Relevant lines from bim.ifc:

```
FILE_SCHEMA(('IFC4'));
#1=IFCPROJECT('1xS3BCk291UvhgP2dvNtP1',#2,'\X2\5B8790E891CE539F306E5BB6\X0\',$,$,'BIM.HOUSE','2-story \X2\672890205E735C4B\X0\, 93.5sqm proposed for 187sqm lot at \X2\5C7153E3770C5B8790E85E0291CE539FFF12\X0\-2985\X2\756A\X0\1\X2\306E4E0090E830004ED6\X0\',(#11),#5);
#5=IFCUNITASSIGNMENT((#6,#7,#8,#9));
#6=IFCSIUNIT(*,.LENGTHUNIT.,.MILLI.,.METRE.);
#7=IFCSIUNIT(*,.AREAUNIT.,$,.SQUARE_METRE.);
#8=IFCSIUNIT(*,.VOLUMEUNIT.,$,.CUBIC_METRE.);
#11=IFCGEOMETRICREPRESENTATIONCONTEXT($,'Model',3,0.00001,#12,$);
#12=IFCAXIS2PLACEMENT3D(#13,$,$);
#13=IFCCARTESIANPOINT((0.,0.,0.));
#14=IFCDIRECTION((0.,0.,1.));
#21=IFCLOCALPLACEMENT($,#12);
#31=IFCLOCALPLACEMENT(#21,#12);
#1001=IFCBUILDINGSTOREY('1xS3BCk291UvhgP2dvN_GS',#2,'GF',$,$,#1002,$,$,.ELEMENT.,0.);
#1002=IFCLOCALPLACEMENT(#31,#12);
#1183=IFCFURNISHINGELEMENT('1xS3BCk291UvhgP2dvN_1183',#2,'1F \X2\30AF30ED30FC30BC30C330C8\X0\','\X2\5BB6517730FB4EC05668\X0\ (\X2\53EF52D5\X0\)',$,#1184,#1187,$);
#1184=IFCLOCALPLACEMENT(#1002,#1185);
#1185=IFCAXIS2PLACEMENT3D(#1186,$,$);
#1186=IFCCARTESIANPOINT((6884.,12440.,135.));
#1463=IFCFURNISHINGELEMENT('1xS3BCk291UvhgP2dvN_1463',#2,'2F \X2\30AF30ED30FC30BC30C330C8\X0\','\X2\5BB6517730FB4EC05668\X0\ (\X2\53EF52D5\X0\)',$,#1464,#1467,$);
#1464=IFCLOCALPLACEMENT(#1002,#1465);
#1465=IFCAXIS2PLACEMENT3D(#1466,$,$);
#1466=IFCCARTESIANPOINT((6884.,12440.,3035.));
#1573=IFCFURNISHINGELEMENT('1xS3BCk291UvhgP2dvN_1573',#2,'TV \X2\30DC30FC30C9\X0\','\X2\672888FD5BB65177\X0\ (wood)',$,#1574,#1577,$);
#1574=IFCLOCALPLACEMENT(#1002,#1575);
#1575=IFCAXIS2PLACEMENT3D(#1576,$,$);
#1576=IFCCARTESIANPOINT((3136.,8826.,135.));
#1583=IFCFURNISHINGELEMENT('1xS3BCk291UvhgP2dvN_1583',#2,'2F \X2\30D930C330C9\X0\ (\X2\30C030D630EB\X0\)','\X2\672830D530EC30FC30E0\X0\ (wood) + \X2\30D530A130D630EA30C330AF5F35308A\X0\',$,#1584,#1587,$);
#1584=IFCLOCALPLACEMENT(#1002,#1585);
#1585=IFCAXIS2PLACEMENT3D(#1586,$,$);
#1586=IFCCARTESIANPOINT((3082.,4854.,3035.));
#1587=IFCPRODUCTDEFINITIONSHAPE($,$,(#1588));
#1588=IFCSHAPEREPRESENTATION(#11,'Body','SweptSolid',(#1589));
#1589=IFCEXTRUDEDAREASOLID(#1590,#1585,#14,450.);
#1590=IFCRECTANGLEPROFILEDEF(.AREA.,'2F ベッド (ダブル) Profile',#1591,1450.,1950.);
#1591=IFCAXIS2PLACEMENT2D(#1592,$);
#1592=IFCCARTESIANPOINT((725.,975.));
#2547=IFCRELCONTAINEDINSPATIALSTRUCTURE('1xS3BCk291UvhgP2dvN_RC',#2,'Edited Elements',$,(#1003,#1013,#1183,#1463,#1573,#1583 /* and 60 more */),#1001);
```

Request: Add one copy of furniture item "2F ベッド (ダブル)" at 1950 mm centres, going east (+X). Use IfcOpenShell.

```python
import numpy as np
import ifcopenshell
import ifcopenshell.api.geometry
import ifcopenshell.api.root
import ifcopenshell.util.element
import ifcopenshell.util.placement

model = ifcopenshell.open("bim.ifc")


def reuse_history(source, copy):
    """copy_class also copies each property set's owner history, people and application; keep the originals."""
    for rel in copy.IsDefinedBy:
        if rel.is_a("IfcRelDefinesByProperties") and (history := rel.RelatingPropertyDefinition.OwnerHistory):
            rel.RelatingPropertyDefinition.OwnerHistory = source.OwnerHistory
            ifcopenshell.util.element.remove_deep2(model, history)


source = model.by_guid("1xS3BCk291UvhgP2dvN_1583")
base = ifcopenshell.util.placement.get_local_placement(source.ObjectPlacement)
step = np.array([1.0, 0.0, 0.0]) * 1950.0

for i in range(1, 2):
    copy = ifcopenshell.api.root.copy_class(model, product=source)
    copy.Representation = ifcopenshell.util.element.copy_deep(
        model, source.Representation, exclude=["IfcGeometricRepresentationContext", "IfcRepresentationMap"]
    )
    reuse_history(source, copy)
    matrix = base.copy()
    matrix[:3, 3] += i * step
    print("added at", matrix[:3, 3].round(3) + 0.0)
    ifcopenshell.api.geometry.edit_object_placement(model, product=copy, matrix=matrix, is_si=False)

model.write("bim-out.ifc")
```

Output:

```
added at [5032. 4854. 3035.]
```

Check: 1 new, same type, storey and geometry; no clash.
